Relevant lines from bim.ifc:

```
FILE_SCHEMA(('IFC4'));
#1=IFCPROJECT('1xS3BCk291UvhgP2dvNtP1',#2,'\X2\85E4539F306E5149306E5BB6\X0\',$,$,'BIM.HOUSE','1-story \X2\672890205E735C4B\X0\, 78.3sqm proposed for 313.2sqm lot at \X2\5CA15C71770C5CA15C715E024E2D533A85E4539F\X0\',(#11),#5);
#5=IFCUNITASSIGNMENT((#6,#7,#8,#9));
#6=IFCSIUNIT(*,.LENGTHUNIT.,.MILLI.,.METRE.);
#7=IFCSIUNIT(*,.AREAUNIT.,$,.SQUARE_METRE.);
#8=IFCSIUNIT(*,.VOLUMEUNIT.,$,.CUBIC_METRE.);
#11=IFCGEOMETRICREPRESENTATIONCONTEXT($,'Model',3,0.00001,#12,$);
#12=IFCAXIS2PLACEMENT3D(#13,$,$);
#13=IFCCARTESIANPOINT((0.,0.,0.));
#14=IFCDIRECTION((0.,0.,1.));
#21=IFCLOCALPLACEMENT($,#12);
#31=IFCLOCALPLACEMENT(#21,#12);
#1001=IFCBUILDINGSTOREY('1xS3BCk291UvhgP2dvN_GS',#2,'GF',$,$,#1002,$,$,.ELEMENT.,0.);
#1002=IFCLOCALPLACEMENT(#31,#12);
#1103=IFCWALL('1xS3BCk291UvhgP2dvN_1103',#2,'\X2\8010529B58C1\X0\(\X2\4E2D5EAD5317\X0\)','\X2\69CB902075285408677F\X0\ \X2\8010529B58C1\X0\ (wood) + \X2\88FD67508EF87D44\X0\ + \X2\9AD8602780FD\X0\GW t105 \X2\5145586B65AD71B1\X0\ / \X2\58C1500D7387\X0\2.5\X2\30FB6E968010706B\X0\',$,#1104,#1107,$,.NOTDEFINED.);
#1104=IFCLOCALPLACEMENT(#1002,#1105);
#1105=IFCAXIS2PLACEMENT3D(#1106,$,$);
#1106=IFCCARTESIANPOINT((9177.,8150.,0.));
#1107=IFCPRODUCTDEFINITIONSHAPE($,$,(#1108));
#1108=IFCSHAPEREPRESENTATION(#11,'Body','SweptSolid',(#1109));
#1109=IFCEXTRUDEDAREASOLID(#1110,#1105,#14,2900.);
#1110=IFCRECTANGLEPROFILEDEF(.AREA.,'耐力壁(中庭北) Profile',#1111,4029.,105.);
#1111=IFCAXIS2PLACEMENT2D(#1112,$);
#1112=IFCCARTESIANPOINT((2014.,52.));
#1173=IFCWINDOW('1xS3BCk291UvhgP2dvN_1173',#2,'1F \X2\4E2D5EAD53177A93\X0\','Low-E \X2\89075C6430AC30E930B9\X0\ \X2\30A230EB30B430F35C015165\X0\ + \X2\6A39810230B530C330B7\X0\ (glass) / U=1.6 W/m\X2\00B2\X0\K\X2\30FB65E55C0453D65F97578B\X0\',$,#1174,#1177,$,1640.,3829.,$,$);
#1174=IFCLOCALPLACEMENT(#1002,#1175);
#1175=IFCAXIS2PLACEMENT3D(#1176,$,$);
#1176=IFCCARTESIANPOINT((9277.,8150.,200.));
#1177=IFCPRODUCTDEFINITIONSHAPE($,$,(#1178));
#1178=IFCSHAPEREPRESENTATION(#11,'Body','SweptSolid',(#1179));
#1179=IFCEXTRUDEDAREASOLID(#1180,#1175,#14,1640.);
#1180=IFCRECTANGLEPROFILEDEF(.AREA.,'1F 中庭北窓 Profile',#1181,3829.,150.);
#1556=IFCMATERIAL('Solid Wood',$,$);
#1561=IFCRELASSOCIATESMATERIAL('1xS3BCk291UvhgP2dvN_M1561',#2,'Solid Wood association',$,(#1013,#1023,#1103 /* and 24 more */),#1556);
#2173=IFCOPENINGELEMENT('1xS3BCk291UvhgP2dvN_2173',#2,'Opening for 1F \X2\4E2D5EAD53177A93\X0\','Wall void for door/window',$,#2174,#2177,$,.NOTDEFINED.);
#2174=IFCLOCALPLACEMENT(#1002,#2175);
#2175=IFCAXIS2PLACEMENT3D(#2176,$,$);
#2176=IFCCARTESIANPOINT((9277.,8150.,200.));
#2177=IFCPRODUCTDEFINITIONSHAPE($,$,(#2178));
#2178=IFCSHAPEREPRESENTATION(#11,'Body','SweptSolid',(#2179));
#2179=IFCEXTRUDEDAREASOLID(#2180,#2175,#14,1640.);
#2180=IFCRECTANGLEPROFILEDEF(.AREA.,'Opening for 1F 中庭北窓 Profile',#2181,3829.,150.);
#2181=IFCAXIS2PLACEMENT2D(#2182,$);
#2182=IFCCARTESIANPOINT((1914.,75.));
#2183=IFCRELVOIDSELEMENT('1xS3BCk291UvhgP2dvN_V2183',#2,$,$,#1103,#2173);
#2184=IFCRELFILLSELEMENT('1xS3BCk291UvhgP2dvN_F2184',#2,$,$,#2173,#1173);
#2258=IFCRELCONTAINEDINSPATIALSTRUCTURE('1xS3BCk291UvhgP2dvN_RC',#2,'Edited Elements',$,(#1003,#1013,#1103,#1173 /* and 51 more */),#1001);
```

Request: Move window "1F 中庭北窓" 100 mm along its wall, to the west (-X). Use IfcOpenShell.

```python
import ifcopenshell
import ifcopenshell.api.geometry
import ifcopenshell.util.placement

model = ifcopenshell.open("bim.ifc")

window = model.by_id(1173)
opening = window.FillsVoids[0].RelatingOpeningElement
wall = opening.VoidsElements[0].RelatingBuildingElement

wall_matrix = ifcopenshell.util.placement.get_local_placement(wall.ObjectPlacement)
shift = wall_matrix[:3, 0] * -100.0
before = ifcopenshell.util.placement.get_local_placement(window.ObjectPlacement)[:3, 3].copy()

# The window is not placed relative to its opening, so move both.
for product in (opening, window):
    matrix = ifcopenshell.util.placement.get_local_placement(product.ObjectPlacement)
    matrix[:3, 3] += shift
    ifcopenshell.api.geometry.edit_object_placement(model, product=product, matrix=matrix, is_si=False)

after = ifcopenshell.util.placement.get_local_placement(window.ObjectPlacement)[:3, 3]
print("window moved by", (after - before).round(3) + 0.0)

model.write("bim_v2.ifc")
```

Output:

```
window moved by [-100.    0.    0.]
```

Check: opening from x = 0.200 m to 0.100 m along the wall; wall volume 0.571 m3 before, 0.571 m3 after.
